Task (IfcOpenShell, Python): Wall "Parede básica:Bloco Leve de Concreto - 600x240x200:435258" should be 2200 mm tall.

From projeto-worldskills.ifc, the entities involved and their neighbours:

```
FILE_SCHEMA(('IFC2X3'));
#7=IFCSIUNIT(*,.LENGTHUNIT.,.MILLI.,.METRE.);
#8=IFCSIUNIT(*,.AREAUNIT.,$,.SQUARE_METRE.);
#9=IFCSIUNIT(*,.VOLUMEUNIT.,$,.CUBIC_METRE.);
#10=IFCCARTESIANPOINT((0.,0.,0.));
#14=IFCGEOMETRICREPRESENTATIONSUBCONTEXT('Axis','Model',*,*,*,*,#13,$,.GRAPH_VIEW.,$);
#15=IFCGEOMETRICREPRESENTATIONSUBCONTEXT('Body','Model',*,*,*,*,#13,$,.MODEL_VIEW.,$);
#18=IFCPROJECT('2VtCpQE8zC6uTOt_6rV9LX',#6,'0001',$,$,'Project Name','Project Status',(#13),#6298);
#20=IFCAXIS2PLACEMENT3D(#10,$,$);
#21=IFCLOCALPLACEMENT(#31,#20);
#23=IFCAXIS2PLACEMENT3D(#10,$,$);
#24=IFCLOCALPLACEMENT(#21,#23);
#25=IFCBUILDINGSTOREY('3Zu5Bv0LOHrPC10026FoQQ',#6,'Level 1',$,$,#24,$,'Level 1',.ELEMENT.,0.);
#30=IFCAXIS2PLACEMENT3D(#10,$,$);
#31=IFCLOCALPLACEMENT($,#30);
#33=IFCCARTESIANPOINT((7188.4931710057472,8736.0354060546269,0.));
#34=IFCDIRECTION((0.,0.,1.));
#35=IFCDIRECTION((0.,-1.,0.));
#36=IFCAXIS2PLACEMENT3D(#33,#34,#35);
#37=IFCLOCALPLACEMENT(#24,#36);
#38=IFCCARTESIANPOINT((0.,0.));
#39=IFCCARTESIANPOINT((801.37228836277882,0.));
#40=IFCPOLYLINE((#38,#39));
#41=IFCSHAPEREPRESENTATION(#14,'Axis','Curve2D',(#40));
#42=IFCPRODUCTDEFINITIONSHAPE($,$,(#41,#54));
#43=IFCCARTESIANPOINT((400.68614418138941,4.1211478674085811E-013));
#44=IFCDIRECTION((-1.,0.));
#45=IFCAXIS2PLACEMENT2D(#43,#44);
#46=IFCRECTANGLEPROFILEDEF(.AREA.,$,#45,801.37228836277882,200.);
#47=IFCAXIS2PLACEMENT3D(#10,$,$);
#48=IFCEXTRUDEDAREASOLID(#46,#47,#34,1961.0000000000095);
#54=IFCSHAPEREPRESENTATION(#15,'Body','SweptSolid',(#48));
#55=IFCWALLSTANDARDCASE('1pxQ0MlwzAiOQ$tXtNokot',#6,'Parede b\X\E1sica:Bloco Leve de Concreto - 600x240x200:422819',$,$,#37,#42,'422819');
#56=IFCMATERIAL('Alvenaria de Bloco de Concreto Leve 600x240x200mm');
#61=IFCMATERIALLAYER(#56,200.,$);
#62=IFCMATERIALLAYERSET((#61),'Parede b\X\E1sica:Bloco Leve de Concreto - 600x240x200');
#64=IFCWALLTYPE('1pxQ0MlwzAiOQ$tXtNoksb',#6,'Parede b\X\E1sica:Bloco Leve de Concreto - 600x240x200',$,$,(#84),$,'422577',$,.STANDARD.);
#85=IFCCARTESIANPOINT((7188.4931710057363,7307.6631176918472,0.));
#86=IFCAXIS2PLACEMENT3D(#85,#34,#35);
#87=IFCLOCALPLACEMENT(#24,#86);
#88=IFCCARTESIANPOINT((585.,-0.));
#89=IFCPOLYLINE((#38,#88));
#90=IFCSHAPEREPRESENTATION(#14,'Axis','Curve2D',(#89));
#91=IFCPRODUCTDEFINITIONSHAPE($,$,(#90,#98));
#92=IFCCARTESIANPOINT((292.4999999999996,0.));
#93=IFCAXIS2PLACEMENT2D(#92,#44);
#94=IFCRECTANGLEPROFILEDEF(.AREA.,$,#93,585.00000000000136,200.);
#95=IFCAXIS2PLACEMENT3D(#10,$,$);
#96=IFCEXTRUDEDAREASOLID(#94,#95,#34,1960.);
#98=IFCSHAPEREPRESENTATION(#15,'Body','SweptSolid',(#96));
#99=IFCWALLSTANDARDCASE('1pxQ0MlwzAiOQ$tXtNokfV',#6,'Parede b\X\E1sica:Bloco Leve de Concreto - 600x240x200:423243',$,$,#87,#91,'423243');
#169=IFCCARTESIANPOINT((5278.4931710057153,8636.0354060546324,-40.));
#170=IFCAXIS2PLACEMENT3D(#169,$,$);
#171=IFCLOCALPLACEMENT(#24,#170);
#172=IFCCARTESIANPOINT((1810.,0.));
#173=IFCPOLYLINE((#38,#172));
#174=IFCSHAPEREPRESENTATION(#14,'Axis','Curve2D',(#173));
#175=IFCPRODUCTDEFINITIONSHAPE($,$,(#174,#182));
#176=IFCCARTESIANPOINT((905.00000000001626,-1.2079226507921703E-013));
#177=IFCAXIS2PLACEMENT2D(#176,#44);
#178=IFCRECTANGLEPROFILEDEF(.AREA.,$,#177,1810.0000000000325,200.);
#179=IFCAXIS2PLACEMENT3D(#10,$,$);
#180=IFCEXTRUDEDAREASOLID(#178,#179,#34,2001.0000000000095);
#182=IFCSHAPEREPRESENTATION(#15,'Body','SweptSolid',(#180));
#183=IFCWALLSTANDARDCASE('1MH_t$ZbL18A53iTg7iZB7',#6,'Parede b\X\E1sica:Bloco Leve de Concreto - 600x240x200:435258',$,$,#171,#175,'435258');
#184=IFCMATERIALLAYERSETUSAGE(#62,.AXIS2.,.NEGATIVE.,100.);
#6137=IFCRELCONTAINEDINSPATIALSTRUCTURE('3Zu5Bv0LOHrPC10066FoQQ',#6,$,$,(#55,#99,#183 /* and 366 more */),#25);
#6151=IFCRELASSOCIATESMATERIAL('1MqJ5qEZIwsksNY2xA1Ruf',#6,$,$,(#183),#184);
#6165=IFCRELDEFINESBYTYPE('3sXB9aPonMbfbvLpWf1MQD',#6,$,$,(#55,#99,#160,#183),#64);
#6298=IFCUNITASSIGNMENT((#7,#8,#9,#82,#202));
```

```python
import ifcopenshell
import ifcopenshell.geom
import ifcopenshell.util.representation
import ifcopenshell.util.shape
import ifcopenshell.util.unit

model = ifcopenshell.open("projeto-worldskills.ifc")
unit_scale = ifcopenshell.util.unit.calculate_unit_scale(model)
settings = ifcopenshell.geom.settings()


def volume(element):
    """Net volume in cubic metres, openings subtracted."""
    shape = ifcopenshell.geom.create_shape(settings, element)
    return ifcopenshell.util.shape.get_volume(shape.geometry)


wall = model.by_guid("1MH_t$ZbL18A53iTg7iZB7")
before = volume(wall)

body = ifcopenshell.util.representation.get_representation(wall, "Model", "Body")
solid = body.Items[0]
old_height = solid.Depth
solid.Depth = 2.2 / unit_scale
after = volume(wall)

print(f"height {old_height:g} -> {solid.Depth:g}, volume {before:.3f} -> {after:.3f} m3")

model.write("projeto-worldskills_edited.ifc")
```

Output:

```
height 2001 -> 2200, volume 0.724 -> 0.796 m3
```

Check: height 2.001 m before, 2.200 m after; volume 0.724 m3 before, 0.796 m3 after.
